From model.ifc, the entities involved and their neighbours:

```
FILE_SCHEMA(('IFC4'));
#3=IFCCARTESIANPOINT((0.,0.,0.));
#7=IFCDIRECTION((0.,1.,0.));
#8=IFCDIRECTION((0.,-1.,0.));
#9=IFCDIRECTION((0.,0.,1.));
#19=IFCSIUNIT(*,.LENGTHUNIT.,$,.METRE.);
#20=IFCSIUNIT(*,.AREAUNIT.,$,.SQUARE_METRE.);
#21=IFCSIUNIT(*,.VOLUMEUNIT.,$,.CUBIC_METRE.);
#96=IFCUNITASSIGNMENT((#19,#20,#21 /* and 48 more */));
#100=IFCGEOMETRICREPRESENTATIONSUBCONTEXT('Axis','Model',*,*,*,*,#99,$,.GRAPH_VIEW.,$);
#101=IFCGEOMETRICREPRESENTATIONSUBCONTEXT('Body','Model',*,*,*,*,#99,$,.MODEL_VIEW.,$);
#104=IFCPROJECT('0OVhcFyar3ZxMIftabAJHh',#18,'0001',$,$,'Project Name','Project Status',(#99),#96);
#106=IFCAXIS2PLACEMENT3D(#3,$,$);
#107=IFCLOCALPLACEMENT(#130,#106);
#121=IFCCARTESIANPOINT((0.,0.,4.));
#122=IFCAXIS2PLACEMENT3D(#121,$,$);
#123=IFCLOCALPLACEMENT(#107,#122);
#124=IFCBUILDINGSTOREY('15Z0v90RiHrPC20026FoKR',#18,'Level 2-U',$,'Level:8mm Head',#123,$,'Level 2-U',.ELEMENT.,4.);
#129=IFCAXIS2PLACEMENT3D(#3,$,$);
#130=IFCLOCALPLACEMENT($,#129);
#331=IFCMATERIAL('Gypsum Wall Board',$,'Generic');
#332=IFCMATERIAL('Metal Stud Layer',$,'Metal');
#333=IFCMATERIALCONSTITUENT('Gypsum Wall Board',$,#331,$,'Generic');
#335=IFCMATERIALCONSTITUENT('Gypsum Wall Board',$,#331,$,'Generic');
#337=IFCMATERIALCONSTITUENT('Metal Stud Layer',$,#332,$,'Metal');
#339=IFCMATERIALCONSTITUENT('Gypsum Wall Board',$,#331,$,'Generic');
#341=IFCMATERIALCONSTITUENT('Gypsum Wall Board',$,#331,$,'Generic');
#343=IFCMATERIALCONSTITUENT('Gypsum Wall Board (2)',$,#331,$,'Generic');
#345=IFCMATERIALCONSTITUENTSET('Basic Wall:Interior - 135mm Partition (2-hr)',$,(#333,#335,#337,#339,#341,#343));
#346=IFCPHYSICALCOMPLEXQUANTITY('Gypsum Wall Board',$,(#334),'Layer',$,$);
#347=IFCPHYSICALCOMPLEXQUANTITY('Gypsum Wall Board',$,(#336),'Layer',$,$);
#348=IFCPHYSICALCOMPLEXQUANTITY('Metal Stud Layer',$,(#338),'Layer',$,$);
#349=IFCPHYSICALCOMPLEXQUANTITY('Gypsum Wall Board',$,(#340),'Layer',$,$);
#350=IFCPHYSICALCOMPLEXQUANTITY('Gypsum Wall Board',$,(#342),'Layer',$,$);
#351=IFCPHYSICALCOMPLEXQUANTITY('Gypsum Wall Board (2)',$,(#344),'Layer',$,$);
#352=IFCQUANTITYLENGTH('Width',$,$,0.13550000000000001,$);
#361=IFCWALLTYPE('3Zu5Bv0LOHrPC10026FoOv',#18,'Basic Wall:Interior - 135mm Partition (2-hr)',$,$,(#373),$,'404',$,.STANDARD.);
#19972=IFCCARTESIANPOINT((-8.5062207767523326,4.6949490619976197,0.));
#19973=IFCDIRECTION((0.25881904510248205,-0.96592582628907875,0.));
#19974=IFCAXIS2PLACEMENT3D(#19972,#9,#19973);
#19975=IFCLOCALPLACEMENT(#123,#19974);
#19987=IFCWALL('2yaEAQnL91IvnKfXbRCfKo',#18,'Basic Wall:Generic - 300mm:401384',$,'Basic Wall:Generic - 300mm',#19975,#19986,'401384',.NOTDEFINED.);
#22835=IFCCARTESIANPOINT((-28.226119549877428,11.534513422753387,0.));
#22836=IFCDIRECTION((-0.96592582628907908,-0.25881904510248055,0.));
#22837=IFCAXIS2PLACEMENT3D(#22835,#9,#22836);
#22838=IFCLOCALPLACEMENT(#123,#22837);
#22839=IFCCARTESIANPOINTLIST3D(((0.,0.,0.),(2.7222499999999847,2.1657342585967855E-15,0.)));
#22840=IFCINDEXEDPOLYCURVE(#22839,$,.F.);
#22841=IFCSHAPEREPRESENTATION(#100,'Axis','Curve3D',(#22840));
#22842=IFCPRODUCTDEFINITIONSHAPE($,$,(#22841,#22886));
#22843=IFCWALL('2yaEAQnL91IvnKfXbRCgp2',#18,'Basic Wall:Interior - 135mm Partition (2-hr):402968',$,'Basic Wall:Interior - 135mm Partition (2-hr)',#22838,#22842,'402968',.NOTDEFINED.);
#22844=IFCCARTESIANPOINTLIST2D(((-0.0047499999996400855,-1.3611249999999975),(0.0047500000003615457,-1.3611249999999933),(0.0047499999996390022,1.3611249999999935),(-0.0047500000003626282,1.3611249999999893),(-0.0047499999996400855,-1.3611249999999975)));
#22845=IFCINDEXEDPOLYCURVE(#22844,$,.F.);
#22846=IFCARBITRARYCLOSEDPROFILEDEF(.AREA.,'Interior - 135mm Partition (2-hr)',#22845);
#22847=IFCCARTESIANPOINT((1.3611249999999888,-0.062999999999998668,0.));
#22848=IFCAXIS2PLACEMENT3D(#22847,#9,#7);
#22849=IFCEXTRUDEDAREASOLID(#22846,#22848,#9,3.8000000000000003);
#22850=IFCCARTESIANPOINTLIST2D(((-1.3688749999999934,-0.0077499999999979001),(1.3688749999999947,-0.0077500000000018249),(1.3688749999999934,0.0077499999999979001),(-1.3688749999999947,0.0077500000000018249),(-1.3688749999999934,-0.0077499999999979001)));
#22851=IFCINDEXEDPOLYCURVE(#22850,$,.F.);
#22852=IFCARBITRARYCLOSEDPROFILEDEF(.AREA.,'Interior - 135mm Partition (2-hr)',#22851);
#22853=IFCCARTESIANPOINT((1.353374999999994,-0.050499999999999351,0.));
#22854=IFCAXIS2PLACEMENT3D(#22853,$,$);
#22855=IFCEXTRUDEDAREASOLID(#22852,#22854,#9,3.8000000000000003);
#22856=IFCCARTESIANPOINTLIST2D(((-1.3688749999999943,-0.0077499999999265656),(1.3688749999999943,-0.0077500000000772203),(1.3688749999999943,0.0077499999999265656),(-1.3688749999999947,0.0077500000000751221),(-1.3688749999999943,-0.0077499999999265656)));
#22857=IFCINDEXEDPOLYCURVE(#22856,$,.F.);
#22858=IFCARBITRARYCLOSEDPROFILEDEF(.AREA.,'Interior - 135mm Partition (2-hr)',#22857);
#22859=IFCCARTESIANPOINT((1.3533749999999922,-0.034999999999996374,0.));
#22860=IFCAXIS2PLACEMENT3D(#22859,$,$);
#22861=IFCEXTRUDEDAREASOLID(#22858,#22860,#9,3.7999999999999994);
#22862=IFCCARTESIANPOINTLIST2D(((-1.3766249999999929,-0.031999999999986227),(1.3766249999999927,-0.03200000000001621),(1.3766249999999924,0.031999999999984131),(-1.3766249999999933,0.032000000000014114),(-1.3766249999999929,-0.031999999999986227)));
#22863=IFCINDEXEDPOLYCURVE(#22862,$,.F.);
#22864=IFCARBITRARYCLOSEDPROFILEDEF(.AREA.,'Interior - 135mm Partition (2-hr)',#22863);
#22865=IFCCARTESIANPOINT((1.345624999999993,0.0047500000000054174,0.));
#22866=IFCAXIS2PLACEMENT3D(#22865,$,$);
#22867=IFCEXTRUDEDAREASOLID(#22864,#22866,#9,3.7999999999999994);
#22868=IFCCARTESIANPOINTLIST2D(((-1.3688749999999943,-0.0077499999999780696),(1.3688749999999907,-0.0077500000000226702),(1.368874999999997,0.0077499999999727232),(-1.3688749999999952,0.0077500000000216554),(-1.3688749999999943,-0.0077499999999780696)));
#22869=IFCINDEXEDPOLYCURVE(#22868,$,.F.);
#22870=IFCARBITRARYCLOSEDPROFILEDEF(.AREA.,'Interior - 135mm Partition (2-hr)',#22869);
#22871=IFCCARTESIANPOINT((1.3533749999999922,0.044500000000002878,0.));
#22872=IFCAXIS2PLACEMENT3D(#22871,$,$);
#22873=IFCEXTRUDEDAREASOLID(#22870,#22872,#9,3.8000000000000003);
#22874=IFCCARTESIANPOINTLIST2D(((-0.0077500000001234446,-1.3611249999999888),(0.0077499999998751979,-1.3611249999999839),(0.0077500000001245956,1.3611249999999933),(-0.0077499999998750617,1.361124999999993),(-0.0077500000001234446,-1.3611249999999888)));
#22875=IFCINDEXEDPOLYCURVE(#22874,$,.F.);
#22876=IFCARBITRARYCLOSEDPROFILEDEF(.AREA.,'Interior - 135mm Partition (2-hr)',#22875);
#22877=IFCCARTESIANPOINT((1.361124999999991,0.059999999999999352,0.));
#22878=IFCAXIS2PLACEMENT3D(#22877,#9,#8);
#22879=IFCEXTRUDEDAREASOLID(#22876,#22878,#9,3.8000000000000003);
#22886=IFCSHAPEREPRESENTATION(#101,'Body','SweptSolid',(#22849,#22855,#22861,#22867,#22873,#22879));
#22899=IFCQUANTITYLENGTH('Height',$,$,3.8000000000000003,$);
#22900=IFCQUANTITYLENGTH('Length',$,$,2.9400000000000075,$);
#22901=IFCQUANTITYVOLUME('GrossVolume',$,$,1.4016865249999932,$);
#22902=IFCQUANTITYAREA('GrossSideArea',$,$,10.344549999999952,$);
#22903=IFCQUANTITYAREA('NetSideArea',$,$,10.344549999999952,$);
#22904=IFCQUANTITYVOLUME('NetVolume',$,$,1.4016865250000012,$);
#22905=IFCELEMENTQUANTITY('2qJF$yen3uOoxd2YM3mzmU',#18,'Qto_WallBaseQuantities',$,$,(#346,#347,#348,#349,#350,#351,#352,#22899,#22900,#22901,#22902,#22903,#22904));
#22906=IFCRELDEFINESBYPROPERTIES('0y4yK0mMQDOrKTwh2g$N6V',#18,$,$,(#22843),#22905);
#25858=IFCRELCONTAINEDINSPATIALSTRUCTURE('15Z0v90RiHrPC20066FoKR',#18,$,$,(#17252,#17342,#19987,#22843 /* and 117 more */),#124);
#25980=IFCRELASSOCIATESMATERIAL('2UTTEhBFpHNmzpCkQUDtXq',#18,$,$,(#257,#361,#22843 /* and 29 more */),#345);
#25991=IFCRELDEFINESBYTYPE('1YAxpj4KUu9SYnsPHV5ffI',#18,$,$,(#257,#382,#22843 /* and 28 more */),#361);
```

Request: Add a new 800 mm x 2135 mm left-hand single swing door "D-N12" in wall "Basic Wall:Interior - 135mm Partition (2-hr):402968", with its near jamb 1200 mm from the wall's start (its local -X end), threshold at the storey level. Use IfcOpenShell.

```python
import numpy as np
import ifcopenshell
import ifcopenshell.api.feature
import ifcopenshell.api.geometry
import ifcopenshell.api.pset
import ifcopenshell.api.root
import ifcopenshell.api.spatial
import ifcopenshell.geom
import ifcopenshell.util.element
import ifcopenshell.util.placement
import ifcopenshell.util.representation
import ifcopenshell.util.shape
import ifcopenshell.util.unit

model = ifcopenshell.open("model.ifc")
unit_scale = ifcopenshell.util.unit.calculate_unit_scale(model)
area_scale = ifcopenshell.util.unit.calculate_unit_scale(model, "AREAUNIT")
volume_scale = ifcopenshell.util.unit.calculate_unit_scale(model, "VOLUMEUNIT")
settings = ifcopenshell.geom.settings()


def volume(element):
    """Net volume in cubic metres, openings subtracted."""
    shape = ifcopenshell.geom.create_shape(settings, element)
    return ifcopenshell.util.shape.get_volume(shape.geometry)


wall = model.by_id(22843)
storey = ifcopenshell.util.element.get_container(wall, ifc_class="IfcBuildingStorey")
context = ifcopenshell.util.representation.get_context(model, "Model", "Body", "MODEL_VIEW")
before = volume(wall)

width, height, from_end, sill = 0.8, 2.135, 1.2, 0.0  # metres

# The wall runs along its own X axis, and the end named is its -X end.
wall_shape = ifcopenshell.geom.create_shape(settings, wall)
x, y, z = ifcopenshell.util.shape.get_vertices(wall_shape.geometry).T
start = x.min() + from_end
face, thickness = float(y.min()), float(y.max() - y.min())
wall_matrix = ifcopenshell.util.placement.get_local_placement(wall.ObjectPlacement)
level = ifcopenshell.util.placement.get_local_placement(storey.ObjectPlacement)[2, 3]


def in_wall(x, y):
    """Placement at x, y metres in the wall's axes, at sill height."""
    matrix = wall_matrix.copy()
    matrix[:, 3] = wall_matrix @ np.array([x / unit_scale, y / unit_scale, 0.0, 1.0])
    matrix[2, 3] = level + sill / unit_scale
    return matrix


# Opening: a box that overshoots both wall faces by 50 mm.
opening = ifcopenshell.api.root.create_entity(model, ifc_class="IfcOpeningElement", predefined_type="OPENING")
box = ifcopenshell.api.geometry.add_wall_representation(
    model, context=context, length=width, height=height, thickness=thickness + 0.1
)
ifcopenshell.api.geometry.assign_representation(model, product=opening, representation=box)
ifcopenshell.api.geometry.edit_object_placement(model, product=opening, matrix=in_wall(start, face - 0.05), is_si=False)
ifcopenshell.api.feature.add_feature(model, feature=opening, element=wall)

door = ifcopenshell.api.root.create_entity(model, ifc_class="IfcDoor", name="D-N12", predefined_type="DOOR")
door.OverallWidth, door.OverallHeight = width / unit_scale, height / unit_scale
door.OperationType = "SINGLE_SWING_LEFT"
body = ifcopenshell.api.geometry.add_door_representation(
    model,
    context=context,
    overall_width=door.OverallWidth,
    overall_height=door.OverallHeight,
    operation_type="SINGLE_SWING_LEFT",
    lining_properties={"LiningDepth": thickness / unit_scale, "ThresholdDepth": thickness / unit_scale},
)
ifcopenshell.api.geometry.assign_representation(model, product=door, representation=body)
ifcopenshell.api.spatial.assign_container(model, products=[door], relating_structure=storey)
ifcopenshell.api.feature.add_filling(model, opening=opening, element=door)

# The lining spans the wall, so the door starts at the wall face.
ifcopenshell.api.geometry.edit_object_placement(model, product=door, matrix=in_wall(start, face), is_si=False)

after = volume(wall)

# Update the wall's stored quantities.
qto = model.by_id(ifcopenshell.util.element.get_pset(wall, "Qto_WallBaseQuantities", should_inherit=False)["id"])
ifcopenshell.api.pset.edit_qto(model, qto=qto, properties={
    "NetSideArea": after / thickness / area_scale,
    "NetVolume": after / volume_scale,
})

print(f"wall volume {before:.3f} -> {after:.3f} m3")

model.write("model_rev.ifc")
```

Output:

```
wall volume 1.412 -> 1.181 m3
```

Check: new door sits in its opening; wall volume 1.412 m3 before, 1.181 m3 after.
